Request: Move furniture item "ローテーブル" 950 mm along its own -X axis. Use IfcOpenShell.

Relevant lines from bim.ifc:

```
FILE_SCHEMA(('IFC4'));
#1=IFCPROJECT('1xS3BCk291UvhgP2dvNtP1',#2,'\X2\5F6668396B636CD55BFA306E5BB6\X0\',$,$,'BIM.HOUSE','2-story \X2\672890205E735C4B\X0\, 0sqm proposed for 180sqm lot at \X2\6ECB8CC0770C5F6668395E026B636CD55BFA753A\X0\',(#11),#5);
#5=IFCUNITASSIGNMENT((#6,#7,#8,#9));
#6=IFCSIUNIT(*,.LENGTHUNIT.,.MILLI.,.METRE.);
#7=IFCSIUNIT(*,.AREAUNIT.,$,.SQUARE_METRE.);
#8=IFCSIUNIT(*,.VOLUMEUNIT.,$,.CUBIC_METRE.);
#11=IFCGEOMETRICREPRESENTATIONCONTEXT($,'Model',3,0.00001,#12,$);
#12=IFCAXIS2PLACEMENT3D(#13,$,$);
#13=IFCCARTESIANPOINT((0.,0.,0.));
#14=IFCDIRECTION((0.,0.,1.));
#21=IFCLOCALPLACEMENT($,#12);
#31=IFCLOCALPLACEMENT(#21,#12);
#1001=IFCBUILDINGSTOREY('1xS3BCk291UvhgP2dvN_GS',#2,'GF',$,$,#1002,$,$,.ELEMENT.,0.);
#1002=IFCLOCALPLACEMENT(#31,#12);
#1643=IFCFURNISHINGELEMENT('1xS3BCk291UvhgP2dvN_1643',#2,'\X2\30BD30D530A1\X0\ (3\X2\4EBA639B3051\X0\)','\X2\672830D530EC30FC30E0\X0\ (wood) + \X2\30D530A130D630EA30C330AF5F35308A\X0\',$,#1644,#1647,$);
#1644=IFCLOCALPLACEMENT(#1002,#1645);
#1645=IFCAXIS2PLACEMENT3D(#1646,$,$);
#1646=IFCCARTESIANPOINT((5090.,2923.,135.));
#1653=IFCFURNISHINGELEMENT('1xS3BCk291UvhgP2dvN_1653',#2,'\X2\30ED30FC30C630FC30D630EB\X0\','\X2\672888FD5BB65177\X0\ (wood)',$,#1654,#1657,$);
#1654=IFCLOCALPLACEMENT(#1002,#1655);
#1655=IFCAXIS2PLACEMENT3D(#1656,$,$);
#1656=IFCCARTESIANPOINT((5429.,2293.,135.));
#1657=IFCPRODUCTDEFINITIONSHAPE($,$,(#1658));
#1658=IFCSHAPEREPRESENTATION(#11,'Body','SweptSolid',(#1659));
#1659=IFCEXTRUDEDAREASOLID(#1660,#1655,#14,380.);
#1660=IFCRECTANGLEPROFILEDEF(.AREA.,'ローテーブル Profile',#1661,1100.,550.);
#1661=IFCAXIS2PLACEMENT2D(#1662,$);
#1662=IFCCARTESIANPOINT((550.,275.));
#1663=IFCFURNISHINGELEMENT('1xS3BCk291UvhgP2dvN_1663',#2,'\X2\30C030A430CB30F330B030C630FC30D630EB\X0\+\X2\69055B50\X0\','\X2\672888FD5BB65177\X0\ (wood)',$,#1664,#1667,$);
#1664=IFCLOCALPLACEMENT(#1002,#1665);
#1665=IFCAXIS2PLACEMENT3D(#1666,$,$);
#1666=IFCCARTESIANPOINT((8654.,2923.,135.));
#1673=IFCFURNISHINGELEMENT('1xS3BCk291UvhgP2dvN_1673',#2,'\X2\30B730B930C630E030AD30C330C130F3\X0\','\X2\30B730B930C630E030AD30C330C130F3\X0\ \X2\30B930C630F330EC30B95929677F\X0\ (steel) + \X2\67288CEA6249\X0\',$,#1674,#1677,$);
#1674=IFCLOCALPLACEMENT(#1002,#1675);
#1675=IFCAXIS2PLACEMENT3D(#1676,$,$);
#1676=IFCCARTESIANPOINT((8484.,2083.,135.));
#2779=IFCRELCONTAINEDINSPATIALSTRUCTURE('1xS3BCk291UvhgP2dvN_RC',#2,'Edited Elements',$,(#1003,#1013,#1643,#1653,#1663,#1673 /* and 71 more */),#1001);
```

```python
import ifcopenshell
import ifcopenshell.api.geometry
import ifcopenshell.util.placement
import ifcopenshell.util.unit

model = ifcopenshell.open("bim.ifc")
unit_scale = ifcopenshell.util.unit.calculate_unit_scale(model)

item = model.by_guid("1xS3BCk291UvhgP2dvN_1653")
matrix = ifcopenshell.util.placement.get_local_placement(item.ObjectPlacement)
matrix[:3, 3] -= matrix[:3, 0] * 0.95 / unit_scale
ifcopenshell.api.geometry.edit_object_placement(model, product=item, matrix=matrix, is_si=False)

print(ifcopenshell.util.placement.get_local_placement(item.ObjectPlacement).round(3) + 0.0)

model.write("bim_updated.ifc")
```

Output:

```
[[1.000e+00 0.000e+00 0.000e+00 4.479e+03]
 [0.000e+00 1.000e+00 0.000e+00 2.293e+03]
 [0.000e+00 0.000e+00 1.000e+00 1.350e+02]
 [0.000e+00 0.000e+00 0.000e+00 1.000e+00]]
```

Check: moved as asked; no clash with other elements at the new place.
